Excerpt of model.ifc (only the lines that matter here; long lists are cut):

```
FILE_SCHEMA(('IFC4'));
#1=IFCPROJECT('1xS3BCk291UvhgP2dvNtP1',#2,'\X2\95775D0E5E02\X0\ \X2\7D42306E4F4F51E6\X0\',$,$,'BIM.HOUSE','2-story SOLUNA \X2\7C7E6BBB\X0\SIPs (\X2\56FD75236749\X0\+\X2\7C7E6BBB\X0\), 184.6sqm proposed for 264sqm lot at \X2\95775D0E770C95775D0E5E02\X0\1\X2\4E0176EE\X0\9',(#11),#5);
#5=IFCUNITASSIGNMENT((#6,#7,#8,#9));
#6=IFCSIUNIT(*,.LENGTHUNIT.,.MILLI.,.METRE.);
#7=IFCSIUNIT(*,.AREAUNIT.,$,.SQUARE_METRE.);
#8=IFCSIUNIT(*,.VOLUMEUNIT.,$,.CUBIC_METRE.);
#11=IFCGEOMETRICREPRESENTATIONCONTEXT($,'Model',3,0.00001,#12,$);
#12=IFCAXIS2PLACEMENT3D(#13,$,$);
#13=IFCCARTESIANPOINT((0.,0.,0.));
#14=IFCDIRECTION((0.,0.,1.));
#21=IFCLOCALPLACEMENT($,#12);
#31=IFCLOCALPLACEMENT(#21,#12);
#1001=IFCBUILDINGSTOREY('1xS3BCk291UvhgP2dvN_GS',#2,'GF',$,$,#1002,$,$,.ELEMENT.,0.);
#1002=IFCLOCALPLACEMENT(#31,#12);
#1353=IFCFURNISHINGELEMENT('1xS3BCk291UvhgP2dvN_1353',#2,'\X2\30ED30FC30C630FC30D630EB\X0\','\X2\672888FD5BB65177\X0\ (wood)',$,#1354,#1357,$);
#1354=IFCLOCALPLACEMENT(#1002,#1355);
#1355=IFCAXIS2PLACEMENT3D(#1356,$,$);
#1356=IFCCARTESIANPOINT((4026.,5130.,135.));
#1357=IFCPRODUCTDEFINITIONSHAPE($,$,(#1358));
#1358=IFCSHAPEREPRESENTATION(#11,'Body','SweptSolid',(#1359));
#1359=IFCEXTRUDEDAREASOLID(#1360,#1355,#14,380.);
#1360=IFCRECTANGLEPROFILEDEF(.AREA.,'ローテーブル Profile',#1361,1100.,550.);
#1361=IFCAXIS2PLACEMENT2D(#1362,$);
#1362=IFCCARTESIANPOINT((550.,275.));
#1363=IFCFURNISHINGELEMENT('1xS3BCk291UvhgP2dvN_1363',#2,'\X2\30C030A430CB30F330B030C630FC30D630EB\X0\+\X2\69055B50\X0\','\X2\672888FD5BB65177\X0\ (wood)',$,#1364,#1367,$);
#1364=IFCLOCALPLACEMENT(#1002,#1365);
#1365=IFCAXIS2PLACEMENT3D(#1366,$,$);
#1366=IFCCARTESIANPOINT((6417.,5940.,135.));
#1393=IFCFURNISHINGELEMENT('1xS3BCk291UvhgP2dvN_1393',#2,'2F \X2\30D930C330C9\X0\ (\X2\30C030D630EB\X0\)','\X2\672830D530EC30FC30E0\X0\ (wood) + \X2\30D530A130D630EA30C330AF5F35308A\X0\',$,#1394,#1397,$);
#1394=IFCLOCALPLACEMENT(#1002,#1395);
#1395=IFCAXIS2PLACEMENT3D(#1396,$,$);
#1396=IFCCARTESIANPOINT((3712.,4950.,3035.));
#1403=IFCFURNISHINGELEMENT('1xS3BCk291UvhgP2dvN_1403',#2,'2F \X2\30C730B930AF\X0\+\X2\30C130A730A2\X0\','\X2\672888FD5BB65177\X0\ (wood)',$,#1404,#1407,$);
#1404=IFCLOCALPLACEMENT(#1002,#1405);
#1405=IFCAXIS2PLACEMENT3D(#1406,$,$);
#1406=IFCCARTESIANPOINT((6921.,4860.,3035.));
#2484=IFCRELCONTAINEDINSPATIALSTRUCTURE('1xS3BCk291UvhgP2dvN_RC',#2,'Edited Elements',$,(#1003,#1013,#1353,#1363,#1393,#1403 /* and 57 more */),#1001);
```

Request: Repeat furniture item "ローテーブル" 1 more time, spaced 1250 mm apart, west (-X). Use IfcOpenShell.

```python
import numpy as np
import ifcopenshell
import ifcopenshell.api.geometry
import ifcopenshell.api.root
import ifcopenshell.util.element
import ifcopenshell.util.placement
import ifcopenshell.util.unit

model = ifcopenshell.open("model.ifc")
unit_scale = ifcopenshell.util.unit.calculate_unit_scale(model)


def reuse_history(source, copy):
    """copy_class also copies each property set's owner history, people and application; keep the originals."""
    for rel in copy.IsDefinedBy:
        if rel.is_a("IfcRelDefinesByProperties") and (history := rel.RelatingPropertyDefinition.OwnerHistory):
            rel.RelatingPropertyDefinition.OwnerHistory = source.OwnerHistory
            ifcopenshell.util.element.remove_deep2(model, history)


source = model.by_id(1353)
base = ifcopenshell.util.placement.get_local_placement(source.ObjectPlacement)
step = np.array([-1.0, 0.0, 0.0]) * 1.25 / unit_scale

for i in range(1, 2):
    copy = ifcopenshell.api.root.copy_class(model, product=source)
    copy.Representation = ifcopenshell.util.element.copy_deep(
        model, source.Representation, exclude=["IfcGeometricRepresentationContext", "IfcRepresentationMap"]
    )
    reuse_history(source, copy)
    matrix = base.copy()
    matrix[:3, 3] += i * step
    print("added at", matrix[:3, 3].round(3) + 0.0)
    ifcopenshell.api.geometry.edit_object_placement(model, product=copy, matrix=matrix, is_si=False)

model.write("model_updated.ifc")
```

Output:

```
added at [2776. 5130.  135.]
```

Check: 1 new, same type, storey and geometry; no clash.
